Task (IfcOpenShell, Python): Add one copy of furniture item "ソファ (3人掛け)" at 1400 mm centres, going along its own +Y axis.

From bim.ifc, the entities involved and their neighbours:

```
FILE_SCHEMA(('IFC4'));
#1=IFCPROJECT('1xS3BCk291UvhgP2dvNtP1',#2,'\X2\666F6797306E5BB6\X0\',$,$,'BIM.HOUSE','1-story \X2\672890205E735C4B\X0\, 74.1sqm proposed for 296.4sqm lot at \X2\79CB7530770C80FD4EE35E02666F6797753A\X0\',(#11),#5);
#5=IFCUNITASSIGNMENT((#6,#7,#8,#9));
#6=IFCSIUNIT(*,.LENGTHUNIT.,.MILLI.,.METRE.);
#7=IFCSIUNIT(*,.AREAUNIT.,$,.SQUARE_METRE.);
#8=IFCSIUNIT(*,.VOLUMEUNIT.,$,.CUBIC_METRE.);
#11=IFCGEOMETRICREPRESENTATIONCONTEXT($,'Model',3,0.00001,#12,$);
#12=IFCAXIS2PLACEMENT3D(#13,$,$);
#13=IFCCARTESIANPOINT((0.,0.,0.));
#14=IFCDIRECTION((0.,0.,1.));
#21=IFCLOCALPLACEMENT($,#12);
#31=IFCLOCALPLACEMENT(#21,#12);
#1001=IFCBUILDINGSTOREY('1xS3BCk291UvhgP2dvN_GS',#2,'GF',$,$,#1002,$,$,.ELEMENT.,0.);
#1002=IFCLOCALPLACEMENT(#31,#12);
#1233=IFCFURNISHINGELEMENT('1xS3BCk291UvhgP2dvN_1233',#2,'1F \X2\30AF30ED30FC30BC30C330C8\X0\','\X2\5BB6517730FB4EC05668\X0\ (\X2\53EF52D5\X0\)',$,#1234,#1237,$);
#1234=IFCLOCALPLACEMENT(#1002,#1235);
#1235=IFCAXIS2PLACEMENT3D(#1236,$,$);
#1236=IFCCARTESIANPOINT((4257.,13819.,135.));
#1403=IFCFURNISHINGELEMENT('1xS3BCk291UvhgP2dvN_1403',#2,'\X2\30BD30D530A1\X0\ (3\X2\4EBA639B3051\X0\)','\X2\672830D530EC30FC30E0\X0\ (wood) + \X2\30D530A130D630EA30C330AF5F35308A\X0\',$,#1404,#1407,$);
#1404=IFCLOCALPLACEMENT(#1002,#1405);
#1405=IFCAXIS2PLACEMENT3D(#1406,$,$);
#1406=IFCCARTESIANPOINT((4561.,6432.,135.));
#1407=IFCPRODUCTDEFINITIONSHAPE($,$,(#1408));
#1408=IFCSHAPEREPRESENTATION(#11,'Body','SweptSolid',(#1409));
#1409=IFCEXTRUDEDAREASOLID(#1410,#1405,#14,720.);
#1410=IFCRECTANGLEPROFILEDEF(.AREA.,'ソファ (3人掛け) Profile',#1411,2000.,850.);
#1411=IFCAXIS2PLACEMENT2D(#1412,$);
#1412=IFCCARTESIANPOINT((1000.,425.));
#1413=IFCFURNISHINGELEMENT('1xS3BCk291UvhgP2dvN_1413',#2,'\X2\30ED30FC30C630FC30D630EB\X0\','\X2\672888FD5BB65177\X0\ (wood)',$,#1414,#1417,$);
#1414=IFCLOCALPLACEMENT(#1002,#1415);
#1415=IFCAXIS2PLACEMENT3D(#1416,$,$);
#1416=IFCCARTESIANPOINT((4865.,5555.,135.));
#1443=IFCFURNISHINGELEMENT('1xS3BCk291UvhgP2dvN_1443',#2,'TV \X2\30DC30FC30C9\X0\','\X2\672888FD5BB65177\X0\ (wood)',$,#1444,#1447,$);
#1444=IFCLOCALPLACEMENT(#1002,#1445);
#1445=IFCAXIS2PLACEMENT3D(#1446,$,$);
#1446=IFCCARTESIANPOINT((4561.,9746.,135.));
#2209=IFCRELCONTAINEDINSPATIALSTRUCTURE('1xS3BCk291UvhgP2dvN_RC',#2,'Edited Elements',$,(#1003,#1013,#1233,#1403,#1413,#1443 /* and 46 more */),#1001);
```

```python
import ifcopenshell
import ifcopenshell.api.geometry
import ifcopenshell.api.root
import ifcopenshell.util.element
import ifcopenshell.util.placement
import ifcopenshell.util.unit

model = ifcopenshell.open("bim.ifc")
unit_scale = ifcopenshell.util.unit.calculate_unit_scale(model)


def reuse_history(source, copy):
    """copy_class also copies each property set's owner history, people and application; keep the originals."""
    for rel in copy.IsDefinedBy:
        if rel.is_a("IfcRelDefinesByProperties") and (history := rel.RelatingPropertyDefinition.OwnerHistory):
            rel.RelatingPropertyDefinition.OwnerHistory = source.OwnerHistory
            ifcopenshell.util.element.remove_deep2(model, history)


source = model.by_guid("1xS3BCk291UvhgP2dvN_1403")
base = ifcopenshell.util.placement.get_local_placement(source.ObjectPlacement)
step = base[:3, 1] * 1.4 / unit_scale

for i in range(1, 2):
    copy = ifcopenshell.api.root.copy_class(model, product=source)
    copy.Representation = ifcopenshell.util.element.copy_deep(
        model, source.Representation, exclude=["IfcGeometricRepresentationContext", "IfcRepresentationMap"]
    )
    reuse_history(source, copy)
    matrix = base.copy()
    matrix[:3, 3] += i * step
    print("added at", matrix[:3, 3].round(3) + 0.0)
    ifcopenshell.api.geometry.edit_object_placement(model, product=copy, matrix=matrix, is_si=False)

model.write("bim_updated.ifc")
```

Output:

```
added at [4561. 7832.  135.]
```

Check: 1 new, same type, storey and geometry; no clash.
